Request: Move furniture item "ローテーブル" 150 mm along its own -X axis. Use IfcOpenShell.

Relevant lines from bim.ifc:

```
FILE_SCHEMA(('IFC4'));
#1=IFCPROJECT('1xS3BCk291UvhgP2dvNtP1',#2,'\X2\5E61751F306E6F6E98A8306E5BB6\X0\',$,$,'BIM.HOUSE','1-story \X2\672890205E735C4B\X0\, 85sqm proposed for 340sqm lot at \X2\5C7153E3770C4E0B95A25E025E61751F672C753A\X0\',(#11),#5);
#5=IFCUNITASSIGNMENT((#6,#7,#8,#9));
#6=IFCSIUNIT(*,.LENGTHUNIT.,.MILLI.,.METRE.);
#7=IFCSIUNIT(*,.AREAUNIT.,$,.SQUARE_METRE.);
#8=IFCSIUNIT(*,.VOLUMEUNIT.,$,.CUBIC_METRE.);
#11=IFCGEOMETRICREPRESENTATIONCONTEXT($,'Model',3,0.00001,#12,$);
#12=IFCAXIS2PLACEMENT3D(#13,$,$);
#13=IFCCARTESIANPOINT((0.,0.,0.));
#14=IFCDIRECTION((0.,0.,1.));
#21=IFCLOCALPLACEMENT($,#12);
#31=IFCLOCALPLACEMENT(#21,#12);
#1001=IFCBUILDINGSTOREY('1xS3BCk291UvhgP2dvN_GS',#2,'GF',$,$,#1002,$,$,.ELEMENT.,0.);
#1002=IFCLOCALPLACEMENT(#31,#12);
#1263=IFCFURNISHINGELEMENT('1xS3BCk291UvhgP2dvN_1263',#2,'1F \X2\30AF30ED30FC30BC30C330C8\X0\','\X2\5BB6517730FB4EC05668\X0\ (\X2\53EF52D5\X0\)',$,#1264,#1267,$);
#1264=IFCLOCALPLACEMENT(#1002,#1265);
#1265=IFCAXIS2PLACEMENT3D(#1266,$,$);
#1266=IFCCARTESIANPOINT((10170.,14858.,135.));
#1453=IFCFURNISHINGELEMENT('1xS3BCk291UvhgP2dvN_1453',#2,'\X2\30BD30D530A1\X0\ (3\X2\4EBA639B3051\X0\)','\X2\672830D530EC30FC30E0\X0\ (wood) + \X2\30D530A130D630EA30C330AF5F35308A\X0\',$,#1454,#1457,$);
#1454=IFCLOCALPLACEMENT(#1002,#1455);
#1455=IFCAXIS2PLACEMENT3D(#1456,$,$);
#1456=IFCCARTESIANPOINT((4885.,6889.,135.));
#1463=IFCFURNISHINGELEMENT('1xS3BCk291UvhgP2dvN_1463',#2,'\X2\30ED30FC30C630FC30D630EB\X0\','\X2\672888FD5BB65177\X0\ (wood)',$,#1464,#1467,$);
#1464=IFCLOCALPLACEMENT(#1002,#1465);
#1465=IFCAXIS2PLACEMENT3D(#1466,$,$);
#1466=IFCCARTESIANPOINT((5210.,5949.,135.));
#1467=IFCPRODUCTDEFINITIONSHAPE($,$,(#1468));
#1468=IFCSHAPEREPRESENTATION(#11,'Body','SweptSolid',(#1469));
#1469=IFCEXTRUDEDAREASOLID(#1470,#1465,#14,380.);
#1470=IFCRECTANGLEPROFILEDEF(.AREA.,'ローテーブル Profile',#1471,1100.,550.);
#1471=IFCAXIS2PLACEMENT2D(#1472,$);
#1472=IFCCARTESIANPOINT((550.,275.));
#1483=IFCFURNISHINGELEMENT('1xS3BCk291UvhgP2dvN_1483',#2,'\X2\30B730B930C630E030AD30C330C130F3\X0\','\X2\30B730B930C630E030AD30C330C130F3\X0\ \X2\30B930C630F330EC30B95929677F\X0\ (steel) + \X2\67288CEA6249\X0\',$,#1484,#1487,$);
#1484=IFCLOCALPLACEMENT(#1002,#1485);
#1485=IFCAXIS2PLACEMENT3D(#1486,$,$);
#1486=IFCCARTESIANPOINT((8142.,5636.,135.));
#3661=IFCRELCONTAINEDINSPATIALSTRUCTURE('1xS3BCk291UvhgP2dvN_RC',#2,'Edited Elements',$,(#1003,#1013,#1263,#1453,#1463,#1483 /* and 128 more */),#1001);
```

```python
import ifcopenshell
import ifcopenshell.api.geometry
import ifcopenshell.util.placement
import ifcopenshell.util.unit

model = ifcopenshell.open("bim.ifc")
unit_scale = ifcopenshell.util.unit.calculate_unit_scale(model)

item = model.by_guid("1xS3BCk291UvhgP2dvN_1463")
matrix = ifcopenshell.util.placement.get_local_placement(item.ObjectPlacement)
matrix[:3, 3] -= matrix[:3, 0] * 0.15 / unit_scale
ifcopenshell.api.geometry.edit_object_placement(model, product=item, matrix=matrix, is_si=False)

print(ifcopenshell.util.placement.get_local_placement(item.ObjectPlacement).round(3) + 0.0)

model.write("bim_edited.ifc")
```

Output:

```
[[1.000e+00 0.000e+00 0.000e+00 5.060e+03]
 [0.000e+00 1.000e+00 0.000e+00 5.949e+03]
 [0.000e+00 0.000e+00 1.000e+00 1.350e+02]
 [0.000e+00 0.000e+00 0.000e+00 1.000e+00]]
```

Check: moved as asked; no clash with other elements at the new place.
